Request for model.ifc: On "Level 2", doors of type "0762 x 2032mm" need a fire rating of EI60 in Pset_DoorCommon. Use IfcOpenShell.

First a look at what the model holds.

```python
import ifcopenshell
import ifcopenshell.util.element

model = ifcopenshell.open("model.ifc")
print(model.schema)
storey = next(s for s in model.by_type("IfcBuildingStorey") if s.Name == "Level 2")
doors = [e for e in ifcopenshell.util.element.get_decomposition(storey) if e.is_a("IfcDoor")]
seen = {}
for e in doors:
    element_type = ifcopenshell.util.element.get_type(e)
    key = (element_type.Name if element_type != e and element_type else None, ifcopenshell.util.element.get_pset(e, "Pset_DoorCommon", "FireRating"))
    seen[key] = seen.get(key, 0) + 1
for (name, value), count in sorted(seen.items(), key=str):
    print(count, "x", name, "|", value)
```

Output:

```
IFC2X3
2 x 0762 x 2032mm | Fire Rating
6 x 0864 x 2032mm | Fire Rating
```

```python
import ifcopenshell
import ifcopenshell.api.pset
import ifcopenshell.util.element

model = ifcopenshell.open("model.ifc")

storey = next(s for s in model.by_type("IfcBuildingStorey") if s.Name == "Level 2")
doors = [e for e in ifcopenshell.util.element.get_decomposition(storey) if e.is_a("IfcDoor")]

count = 0
for e in doors:
    element_type = ifcopenshell.util.element.get_type(e)
    if element_type in (None, e) or element_type.Name != "0762 x 2032mm":
        continue
    # add_pset returns the element's existing set when there is one.
    pset = ifcopenshell.api.pset.add_pset(model, product=e, name="Pset_DoorCommon")
    ifcopenshell.api.pset.edit_pset(model, pset=pset, properties={"FireRating": "EI60"})
    count += 1

print(count, "doors updated")

model.write("model_v2.ifc")
```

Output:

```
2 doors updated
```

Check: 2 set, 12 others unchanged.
